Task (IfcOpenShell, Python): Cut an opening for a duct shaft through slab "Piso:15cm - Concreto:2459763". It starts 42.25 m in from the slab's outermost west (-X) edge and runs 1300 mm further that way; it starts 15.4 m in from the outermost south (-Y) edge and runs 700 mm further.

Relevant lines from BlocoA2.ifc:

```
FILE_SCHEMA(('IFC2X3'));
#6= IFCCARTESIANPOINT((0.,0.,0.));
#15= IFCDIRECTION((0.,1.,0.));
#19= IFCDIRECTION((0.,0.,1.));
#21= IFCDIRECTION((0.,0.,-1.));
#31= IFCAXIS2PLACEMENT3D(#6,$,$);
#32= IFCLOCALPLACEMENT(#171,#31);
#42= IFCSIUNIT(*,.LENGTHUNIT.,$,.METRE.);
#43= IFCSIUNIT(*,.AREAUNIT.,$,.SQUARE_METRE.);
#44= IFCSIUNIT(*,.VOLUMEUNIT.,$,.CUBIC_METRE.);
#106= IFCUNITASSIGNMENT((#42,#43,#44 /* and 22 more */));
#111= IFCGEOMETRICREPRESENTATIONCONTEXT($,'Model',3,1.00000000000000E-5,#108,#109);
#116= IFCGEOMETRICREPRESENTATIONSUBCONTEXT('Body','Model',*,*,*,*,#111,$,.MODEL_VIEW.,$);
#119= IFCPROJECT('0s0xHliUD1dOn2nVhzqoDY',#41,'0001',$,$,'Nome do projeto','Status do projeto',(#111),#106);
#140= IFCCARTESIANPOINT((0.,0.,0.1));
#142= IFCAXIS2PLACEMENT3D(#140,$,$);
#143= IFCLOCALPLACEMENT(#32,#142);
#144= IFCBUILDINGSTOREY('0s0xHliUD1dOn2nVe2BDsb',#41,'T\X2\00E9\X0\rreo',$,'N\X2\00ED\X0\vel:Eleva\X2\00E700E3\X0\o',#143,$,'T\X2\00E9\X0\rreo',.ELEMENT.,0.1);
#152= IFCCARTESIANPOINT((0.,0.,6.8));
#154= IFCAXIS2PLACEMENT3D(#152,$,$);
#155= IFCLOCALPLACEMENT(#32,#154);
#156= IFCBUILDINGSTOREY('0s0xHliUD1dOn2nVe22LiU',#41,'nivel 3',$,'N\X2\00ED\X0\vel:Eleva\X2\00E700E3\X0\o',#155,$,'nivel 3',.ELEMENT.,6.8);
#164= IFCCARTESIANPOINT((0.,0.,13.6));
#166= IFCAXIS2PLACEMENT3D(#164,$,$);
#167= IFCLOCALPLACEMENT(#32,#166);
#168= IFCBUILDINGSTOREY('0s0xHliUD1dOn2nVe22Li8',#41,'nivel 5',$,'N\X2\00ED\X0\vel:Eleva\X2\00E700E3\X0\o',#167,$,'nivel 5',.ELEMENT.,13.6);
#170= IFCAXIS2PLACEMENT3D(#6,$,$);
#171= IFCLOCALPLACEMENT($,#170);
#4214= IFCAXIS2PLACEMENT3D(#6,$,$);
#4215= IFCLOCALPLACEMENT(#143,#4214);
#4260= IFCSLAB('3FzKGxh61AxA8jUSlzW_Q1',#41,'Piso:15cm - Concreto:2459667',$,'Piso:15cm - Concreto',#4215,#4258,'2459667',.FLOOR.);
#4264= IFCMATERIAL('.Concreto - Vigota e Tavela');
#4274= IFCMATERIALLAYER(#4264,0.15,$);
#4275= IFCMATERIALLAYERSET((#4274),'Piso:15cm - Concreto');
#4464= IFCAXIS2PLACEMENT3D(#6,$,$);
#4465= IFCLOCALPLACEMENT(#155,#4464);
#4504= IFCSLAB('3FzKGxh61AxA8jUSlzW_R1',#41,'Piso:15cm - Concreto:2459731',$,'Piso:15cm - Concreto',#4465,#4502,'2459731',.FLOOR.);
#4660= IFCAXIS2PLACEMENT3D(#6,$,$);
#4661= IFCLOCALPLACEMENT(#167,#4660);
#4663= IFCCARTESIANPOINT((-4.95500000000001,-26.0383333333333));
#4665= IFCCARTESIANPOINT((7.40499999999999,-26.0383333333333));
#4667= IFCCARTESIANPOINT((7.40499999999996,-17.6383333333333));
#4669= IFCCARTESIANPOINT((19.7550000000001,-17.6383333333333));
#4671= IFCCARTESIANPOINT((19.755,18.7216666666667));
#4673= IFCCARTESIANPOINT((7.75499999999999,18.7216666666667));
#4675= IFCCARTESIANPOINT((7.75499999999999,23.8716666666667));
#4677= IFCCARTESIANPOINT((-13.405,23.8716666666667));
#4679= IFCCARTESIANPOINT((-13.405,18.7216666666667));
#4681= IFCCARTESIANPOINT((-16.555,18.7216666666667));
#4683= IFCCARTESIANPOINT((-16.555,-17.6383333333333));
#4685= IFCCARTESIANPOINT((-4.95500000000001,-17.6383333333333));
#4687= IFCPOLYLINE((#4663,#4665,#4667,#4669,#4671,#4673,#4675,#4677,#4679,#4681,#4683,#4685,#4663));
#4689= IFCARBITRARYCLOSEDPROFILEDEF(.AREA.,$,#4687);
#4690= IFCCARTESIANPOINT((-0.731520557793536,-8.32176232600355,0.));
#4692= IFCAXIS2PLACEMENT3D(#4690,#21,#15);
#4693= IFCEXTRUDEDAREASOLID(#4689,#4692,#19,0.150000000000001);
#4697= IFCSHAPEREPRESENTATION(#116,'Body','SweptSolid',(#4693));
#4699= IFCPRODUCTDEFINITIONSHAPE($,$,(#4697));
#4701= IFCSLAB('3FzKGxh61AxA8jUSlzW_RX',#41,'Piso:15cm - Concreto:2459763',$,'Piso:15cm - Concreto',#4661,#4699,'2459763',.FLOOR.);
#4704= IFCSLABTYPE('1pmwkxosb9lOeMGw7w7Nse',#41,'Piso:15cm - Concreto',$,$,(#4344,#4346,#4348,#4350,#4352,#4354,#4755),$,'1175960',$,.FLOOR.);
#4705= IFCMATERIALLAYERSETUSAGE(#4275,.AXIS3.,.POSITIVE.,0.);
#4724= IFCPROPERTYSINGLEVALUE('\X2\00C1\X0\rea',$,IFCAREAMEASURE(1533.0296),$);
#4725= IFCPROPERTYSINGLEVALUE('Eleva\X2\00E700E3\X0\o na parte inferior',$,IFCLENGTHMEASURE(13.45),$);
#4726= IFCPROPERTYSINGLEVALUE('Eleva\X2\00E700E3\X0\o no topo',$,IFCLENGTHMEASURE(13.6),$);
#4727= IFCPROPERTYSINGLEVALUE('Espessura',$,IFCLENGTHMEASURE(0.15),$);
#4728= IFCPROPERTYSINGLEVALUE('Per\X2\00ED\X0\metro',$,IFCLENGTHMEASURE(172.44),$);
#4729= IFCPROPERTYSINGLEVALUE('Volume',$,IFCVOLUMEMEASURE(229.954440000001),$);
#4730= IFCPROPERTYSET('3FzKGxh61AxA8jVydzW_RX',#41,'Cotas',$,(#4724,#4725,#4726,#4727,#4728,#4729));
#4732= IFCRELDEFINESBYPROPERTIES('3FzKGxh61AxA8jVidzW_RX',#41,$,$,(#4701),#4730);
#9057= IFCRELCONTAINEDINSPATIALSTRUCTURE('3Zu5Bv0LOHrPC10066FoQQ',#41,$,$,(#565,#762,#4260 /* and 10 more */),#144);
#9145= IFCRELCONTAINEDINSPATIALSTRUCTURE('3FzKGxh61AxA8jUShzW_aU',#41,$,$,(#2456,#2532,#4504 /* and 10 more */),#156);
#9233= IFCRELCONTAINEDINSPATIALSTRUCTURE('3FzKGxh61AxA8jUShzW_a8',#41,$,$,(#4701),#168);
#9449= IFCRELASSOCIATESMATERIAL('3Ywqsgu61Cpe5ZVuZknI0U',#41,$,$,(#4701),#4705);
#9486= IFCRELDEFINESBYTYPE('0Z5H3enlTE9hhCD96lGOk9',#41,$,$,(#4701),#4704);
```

```python
import numpy as np
import ifcopenshell
import ifcopenshell.api.feature
import ifcopenshell.api.geometry
import ifcopenshell.api.pset
import ifcopenshell.api.root
import ifcopenshell.geom
import ifcopenshell.util.element
import ifcopenshell.util.placement
import ifcopenshell.util.representation
import ifcopenshell.util.shape
import ifcopenshell.util.unit

model = ifcopenshell.open("BlocoA2.ifc")
unit_scale = ifcopenshell.util.unit.calculate_unit_scale(model)
area_scale = ifcopenshell.util.unit.calculate_unit_scale(model, "AREAUNIT")
volume_scale = ifcopenshell.util.unit.calculate_unit_scale(model, "VOLUMEUNIT")
settings = ifcopenshell.geom.settings()


def volume(element):
    """Net volume in cubic metres, openings subtracted."""
    shape = ifcopenshell.geom.create_shape(settings, element)
    return ifcopenshell.util.shape.get_volume(shape.geometry)


slab = model.by_id(4701)
before = volume(slab)

# Extent in the slab's own axes, in metres. The edges named are its -X and -Y sides.
slab_shape = ifcopenshell.geom.create_shape(settings, slab)
vertices = ifcopenshell.util.shape.get_vertices(slab_shape.geometry)
x_min, y_min, bottom = vertices.min(axis=0)
top = vertices[:, 2].max()

opening = ifcopenshell.api.root.create_entity(model, ifc_class="IfcOpeningElement", name="Duct shaft opening")
context = ifcopenshell.util.representation.get_context(model, "Model", "Body", "MODEL_VIEW")
width, depth = 1.3, 0.7
outline = [(0.0, 0.0), (width, 0.0), (width, depth), (0.0, depth), (0.0, 0.0)]
# Overshoot both faces by 50 mm so the cut is clean.
shape = ifcopenshell.api.geometry.add_slab_representation(
    model, context=context, depth=top - bottom + 0.1, polyline=outline
)
ifcopenshell.api.geometry.assign_representation(model, product=opening, representation=shape)

matrix = ifcopenshell.util.placement.get_local_placement(slab.ObjectPlacement)
matrix[:, 3] = matrix @ np.append(np.array([x_min + 42.25, y_min + 15.4, bottom - 0.05]) / unit_scale, 1.0)
ifcopenshell.api.geometry.edit_object_placement(model, product=opening, matrix=matrix, is_si=False)
ifcopenshell.api.feature.add_feature(model, feature=opening, element=slab)

after = volume(slab)

# Update the slab's stored quantities.
pset = model.by_id(ifcopenshell.util.element.get_pset(slab, "Cotas", should_inherit=False)["id"])
ifcopenshell.api.pset.edit_pset(model, pset=pset, properties={
    "Área": model.create_entity("IfcAreaMeasure", after / (top - bottom) / area_scale),
    "Volume": model.create_entity("IfcVolumeMeasure", after / volume_scale),
})

print(f"slab volume {before:.3f} -> {after:.3f} m3")

model.write("BlocoA2_v2.ifc")
```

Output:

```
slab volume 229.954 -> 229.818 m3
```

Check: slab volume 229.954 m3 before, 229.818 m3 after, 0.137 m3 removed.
